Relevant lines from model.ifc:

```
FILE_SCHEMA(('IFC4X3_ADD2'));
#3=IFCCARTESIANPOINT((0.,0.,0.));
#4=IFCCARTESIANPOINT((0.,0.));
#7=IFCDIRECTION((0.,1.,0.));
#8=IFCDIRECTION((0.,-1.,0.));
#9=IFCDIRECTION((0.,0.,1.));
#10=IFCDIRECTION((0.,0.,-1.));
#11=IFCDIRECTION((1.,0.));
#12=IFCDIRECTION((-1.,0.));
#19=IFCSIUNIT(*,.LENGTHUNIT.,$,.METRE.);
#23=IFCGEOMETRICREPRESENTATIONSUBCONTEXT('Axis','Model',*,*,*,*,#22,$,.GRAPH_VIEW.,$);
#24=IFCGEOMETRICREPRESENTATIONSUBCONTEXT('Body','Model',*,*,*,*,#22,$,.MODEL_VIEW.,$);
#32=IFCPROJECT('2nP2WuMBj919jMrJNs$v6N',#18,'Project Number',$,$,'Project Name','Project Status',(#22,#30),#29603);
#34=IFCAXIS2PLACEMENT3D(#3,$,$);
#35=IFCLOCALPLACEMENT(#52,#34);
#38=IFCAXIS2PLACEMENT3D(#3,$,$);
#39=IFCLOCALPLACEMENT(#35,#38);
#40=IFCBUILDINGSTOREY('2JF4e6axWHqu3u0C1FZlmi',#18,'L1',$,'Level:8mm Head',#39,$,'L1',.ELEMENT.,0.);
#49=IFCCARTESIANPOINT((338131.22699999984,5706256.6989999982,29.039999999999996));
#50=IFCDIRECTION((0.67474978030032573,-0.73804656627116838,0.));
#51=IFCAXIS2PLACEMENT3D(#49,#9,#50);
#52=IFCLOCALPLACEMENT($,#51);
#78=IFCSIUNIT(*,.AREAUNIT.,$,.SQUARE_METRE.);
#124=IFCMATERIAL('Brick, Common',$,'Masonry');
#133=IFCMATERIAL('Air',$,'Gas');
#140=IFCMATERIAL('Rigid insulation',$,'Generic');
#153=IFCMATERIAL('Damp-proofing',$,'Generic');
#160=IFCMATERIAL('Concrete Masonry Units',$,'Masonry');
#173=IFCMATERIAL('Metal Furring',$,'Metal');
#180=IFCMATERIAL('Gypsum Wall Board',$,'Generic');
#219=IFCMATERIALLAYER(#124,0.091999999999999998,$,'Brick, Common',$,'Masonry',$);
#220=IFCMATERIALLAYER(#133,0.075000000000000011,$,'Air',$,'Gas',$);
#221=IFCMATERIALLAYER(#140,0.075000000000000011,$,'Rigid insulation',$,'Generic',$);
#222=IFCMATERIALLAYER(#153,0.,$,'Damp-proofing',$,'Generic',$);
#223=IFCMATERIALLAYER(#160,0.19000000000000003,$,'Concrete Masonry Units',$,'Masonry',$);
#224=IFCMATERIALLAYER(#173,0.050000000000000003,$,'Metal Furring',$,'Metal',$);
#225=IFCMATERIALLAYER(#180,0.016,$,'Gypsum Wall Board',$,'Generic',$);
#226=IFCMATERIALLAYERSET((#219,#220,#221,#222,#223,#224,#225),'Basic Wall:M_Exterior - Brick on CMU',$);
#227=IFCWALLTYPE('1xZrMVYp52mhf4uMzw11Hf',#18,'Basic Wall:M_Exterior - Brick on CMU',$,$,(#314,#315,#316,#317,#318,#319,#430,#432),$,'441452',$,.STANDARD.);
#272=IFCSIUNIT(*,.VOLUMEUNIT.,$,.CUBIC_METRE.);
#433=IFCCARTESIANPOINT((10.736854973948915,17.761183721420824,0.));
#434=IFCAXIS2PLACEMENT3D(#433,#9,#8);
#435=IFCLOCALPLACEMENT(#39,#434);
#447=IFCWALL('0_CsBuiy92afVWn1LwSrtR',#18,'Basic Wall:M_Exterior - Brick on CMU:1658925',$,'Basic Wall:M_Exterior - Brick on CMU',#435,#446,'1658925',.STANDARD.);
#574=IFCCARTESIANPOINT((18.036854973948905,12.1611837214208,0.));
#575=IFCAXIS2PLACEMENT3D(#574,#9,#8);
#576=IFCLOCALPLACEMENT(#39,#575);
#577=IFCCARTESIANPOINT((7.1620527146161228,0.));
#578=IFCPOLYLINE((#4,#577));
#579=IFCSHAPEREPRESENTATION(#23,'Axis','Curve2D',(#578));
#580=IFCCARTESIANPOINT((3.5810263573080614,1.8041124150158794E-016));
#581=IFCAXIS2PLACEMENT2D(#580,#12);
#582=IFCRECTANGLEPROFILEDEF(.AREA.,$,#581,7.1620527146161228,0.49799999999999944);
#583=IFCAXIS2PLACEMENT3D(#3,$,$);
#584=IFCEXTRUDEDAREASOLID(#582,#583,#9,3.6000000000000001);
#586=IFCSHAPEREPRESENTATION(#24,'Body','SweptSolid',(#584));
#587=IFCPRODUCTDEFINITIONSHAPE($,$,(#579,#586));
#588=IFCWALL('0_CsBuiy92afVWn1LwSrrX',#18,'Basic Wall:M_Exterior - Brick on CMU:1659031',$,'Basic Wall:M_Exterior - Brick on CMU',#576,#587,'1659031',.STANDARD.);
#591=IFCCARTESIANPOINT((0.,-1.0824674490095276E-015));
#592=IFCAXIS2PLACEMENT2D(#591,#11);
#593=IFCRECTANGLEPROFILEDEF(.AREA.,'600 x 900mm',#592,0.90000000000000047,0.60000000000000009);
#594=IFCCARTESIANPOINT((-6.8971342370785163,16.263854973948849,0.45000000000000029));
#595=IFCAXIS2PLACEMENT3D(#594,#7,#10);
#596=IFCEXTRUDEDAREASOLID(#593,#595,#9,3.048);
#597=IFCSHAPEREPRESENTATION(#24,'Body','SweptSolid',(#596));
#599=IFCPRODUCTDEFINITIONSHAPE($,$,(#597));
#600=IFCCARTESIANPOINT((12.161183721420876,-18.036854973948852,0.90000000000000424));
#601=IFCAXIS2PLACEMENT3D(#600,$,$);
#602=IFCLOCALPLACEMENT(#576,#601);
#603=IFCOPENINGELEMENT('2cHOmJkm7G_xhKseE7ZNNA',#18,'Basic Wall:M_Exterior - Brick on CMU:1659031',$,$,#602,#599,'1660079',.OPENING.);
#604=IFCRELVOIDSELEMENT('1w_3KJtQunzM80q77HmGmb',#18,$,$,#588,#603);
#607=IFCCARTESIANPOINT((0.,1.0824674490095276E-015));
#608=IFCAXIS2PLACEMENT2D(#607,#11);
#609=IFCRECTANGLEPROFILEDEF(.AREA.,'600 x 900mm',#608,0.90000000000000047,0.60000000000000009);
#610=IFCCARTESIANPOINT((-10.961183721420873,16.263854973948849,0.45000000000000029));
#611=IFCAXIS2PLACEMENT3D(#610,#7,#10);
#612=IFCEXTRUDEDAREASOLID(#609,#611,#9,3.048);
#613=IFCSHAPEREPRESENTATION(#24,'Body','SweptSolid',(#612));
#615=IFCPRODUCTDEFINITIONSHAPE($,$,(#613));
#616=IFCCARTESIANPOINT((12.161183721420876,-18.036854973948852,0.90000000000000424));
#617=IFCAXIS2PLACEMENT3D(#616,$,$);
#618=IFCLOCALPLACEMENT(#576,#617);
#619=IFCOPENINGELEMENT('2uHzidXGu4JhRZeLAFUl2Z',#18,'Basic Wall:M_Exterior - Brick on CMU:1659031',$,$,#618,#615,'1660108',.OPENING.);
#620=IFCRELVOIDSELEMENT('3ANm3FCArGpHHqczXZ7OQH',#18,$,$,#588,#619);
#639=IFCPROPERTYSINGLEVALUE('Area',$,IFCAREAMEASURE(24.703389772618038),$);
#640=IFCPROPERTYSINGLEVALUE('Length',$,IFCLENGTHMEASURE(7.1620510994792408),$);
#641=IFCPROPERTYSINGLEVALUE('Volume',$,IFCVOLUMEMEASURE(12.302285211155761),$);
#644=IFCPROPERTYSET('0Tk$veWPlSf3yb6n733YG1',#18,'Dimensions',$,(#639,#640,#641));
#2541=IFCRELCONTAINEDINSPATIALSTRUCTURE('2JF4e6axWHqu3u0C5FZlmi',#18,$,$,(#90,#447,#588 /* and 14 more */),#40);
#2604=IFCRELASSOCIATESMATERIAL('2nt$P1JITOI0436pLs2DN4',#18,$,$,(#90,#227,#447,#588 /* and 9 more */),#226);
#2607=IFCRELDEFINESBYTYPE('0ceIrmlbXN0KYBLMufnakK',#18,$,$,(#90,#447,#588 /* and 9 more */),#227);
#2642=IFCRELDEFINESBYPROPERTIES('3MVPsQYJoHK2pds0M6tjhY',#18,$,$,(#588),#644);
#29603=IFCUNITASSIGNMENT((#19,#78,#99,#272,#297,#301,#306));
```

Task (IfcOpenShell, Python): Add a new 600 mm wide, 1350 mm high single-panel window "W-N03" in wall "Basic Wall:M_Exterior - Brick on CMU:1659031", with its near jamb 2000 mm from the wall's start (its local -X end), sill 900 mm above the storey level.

```python
import numpy as np
import ifcopenshell
import ifcopenshell.api.feature
import ifcopenshell.api.geometry
import ifcopenshell.api.pset
import ifcopenshell.api.root
import ifcopenshell.api.spatial
import ifcopenshell.geom
import ifcopenshell.util.element
import ifcopenshell.util.placement
import ifcopenshell.util.representation
import ifcopenshell.util.shape
import ifcopenshell.util.unit

model = ifcopenshell.open("model.ifc")
unit_scale = ifcopenshell.util.unit.calculate_unit_scale(model)
area_scale = ifcopenshell.util.unit.calculate_unit_scale(model, "AREAUNIT")
volume_scale = ifcopenshell.util.unit.calculate_unit_scale(model, "VOLUMEUNIT")
settings = ifcopenshell.geom.settings()


def volume(element):
    """Net volume in cubic metres, openings subtracted."""
    shape = ifcopenshell.geom.create_shape(settings, element)
    return ifcopenshell.util.shape.get_volume(shape.geometry)


wall = model.by_id(588)
storey = ifcopenshell.util.element.get_container(wall, ifc_class="IfcBuildingStorey")
context = ifcopenshell.util.representation.get_context(model, "Model", "Body", "MODEL_VIEW")
before = volume(wall)

width, height, from_end, sill = 0.6, 1.35, 2, 0.9  # metres

# The wall runs along its own X axis, and the end named is its -X end.
wall_shape = ifcopenshell.geom.create_shape(settings, wall)
x, y, z = ifcopenshell.util.shape.get_vertices(wall_shape.geometry).T
start = x.min() + from_end
face, thickness = float(y.min()), float(y.max() - y.min())
wall_matrix = ifcopenshell.util.placement.get_local_placement(wall.ObjectPlacement)
level = ifcopenshell.util.placement.get_local_placement(storey.ObjectPlacement)[2, 3]


def in_wall(x, y):
    """Placement at x, y metres in the wall's axes, at sill height."""
    matrix = wall_matrix.copy()
    matrix[:, 3] = wall_matrix @ np.array([x / unit_scale, y / unit_scale, 0.0, 1.0])
    matrix[2, 3] = level + sill / unit_scale
    return matrix


# Opening: a box that overshoots both wall faces by 50 mm.
opening = ifcopenshell.api.root.create_entity(model, ifc_class="IfcOpeningElement", predefined_type="OPENING")
box = ifcopenshell.api.geometry.add_wall_representation(
    model, context=context, length=width, height=height, thickness=thickness + 0.1
)
ifcopenshell.api.geometry.assign_representation(model, product=opening, representation=box)
ifcopenshell.api.geometry.edit_object_placement(model, product=opening, matrix=in_wall(start, face - 0.05), is_si=False)
ifcopenshell.api.feature.add_feature(model, feature=opening, element=wall)

window = ifcopenshell.api.root.create_entity(model, ifc_class="IfcWindow", name="W-N03", predefined_type="WINDOW")
window.OverallWidth, window.OverallHeight = width / unit_scale, height / unit_scale
window.PartitioningType = "SINGLE_PANEL"
body = ifcopenshell.api.geometry.add_window_representation(
    model,
    context=context,
    overall_width=window.OverallWidth,
    overall_height=window.OverallHeight,
    partition_type="SINGLE_PANEL",
)
ifcopenshell.api.geometry.assign_representation(model, product=window, representation=body)
ifcopenshell.api.spatial.assign_container(model, products=[window], relating_structure=storey)
ifcopenshell.api.feature.add_filling(model, opening=opening, element=window)

# Centre the window in the wall's thickness.
ifcopenshell.api.geometry.edit_object_placement(model, product=window, matrix=in_wall(start, face), is_si=False)
window_shape = ifcopenshell.geom.create_shape(settings, window)
depth = ifcopenshell.util.shape.get_vertices(window_shape.geometry)[:, 1]
offset = face + thickness / 2 - (depth.min() + depth.max()) / 2
ifcopenshell.api.geometry.edit_object_placement(model, product=window, matrix=in_wall(start, offset), is_si=False)

after = volume(wall)

# Update the wall's stored quantities.
pset = model.by_id(ifcopenshell.util.element.get_pset(wall, "Dimensions", should_inherit=False)["id"])
ifcopenshell.api.pset.edit_pset(model, pset=pset, properties={
    "Area": model.create_entity("IfcAreaMeasure", after / thickness / area_scale),
    "Volume": model.create_entity("IfcVolumeMeasure", after / volume_scale),
})

print(f"wall volume {before:.3f} -> {after:.3f} m3")

model.write("model_edited.ifc")
```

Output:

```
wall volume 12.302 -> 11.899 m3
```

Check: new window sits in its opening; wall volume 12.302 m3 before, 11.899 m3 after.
